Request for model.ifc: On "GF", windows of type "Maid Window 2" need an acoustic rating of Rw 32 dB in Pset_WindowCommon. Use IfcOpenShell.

First a look at what the model holds.

```python
import ifcopenshell
import ifcopenshell.util.element

model = ifcopenshell.open("model.ifc")
print(model.schema)
storey = next(s for s in model.by_type("IfcBuildingStorey") if s.Name == "GF")
windows = [e for e in ifcopenshell.util.element.get_decomposition(storey) if e.is_a("IfcWindow")]
seen = {}
for e in windows:
    element_type = ifcopenshell.util.element.get_type(e)
    key = (element_type.Name if element_type != e and element_type else None, ifcopenshell.util.element.get_pset(e, "Pset_WindowCommon", "AcousticRating"))
    seen[key] = seen.get(key, 0) + 1
for (name, value), count in sorted(seen.items(), key=str):
    print(count, "x", name, "|", value)
```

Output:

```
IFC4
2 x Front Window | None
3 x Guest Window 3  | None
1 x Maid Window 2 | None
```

```python
import ifcopenshell
import ifcopenshell.api.pset
import ifcopenshell.util.element

model = ifcopenshell.open("model.ifc")

storey = next(s for s in model.by_type("IfcBuildingStorey") if s.Name == "GF")
windows = [e for e in ifcopenshell.util.element.get_decomposition(storey) if e.is_a("IfcWindow")]

count = 0
for e in windows:
    element_type = ifcopenshell.util.element.get_type(e)
    if element_type in (None, e) or element_type.Name != "Maid Window 2":
        continue
    # add_pset returns the element's existing set when there is one.
    pset = ifcopenshell.api.pset.add_pset(model, product=e, name="Pset_WindowCommon")
    ifcopenshell.api.pset.edit_pset(model, pset=pset, properties={"AcousticRating": "Rw 32 dB"})
    count += 1

print(count, "windows updated")

model.write("model-out.ifc")
```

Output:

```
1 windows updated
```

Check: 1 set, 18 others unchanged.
